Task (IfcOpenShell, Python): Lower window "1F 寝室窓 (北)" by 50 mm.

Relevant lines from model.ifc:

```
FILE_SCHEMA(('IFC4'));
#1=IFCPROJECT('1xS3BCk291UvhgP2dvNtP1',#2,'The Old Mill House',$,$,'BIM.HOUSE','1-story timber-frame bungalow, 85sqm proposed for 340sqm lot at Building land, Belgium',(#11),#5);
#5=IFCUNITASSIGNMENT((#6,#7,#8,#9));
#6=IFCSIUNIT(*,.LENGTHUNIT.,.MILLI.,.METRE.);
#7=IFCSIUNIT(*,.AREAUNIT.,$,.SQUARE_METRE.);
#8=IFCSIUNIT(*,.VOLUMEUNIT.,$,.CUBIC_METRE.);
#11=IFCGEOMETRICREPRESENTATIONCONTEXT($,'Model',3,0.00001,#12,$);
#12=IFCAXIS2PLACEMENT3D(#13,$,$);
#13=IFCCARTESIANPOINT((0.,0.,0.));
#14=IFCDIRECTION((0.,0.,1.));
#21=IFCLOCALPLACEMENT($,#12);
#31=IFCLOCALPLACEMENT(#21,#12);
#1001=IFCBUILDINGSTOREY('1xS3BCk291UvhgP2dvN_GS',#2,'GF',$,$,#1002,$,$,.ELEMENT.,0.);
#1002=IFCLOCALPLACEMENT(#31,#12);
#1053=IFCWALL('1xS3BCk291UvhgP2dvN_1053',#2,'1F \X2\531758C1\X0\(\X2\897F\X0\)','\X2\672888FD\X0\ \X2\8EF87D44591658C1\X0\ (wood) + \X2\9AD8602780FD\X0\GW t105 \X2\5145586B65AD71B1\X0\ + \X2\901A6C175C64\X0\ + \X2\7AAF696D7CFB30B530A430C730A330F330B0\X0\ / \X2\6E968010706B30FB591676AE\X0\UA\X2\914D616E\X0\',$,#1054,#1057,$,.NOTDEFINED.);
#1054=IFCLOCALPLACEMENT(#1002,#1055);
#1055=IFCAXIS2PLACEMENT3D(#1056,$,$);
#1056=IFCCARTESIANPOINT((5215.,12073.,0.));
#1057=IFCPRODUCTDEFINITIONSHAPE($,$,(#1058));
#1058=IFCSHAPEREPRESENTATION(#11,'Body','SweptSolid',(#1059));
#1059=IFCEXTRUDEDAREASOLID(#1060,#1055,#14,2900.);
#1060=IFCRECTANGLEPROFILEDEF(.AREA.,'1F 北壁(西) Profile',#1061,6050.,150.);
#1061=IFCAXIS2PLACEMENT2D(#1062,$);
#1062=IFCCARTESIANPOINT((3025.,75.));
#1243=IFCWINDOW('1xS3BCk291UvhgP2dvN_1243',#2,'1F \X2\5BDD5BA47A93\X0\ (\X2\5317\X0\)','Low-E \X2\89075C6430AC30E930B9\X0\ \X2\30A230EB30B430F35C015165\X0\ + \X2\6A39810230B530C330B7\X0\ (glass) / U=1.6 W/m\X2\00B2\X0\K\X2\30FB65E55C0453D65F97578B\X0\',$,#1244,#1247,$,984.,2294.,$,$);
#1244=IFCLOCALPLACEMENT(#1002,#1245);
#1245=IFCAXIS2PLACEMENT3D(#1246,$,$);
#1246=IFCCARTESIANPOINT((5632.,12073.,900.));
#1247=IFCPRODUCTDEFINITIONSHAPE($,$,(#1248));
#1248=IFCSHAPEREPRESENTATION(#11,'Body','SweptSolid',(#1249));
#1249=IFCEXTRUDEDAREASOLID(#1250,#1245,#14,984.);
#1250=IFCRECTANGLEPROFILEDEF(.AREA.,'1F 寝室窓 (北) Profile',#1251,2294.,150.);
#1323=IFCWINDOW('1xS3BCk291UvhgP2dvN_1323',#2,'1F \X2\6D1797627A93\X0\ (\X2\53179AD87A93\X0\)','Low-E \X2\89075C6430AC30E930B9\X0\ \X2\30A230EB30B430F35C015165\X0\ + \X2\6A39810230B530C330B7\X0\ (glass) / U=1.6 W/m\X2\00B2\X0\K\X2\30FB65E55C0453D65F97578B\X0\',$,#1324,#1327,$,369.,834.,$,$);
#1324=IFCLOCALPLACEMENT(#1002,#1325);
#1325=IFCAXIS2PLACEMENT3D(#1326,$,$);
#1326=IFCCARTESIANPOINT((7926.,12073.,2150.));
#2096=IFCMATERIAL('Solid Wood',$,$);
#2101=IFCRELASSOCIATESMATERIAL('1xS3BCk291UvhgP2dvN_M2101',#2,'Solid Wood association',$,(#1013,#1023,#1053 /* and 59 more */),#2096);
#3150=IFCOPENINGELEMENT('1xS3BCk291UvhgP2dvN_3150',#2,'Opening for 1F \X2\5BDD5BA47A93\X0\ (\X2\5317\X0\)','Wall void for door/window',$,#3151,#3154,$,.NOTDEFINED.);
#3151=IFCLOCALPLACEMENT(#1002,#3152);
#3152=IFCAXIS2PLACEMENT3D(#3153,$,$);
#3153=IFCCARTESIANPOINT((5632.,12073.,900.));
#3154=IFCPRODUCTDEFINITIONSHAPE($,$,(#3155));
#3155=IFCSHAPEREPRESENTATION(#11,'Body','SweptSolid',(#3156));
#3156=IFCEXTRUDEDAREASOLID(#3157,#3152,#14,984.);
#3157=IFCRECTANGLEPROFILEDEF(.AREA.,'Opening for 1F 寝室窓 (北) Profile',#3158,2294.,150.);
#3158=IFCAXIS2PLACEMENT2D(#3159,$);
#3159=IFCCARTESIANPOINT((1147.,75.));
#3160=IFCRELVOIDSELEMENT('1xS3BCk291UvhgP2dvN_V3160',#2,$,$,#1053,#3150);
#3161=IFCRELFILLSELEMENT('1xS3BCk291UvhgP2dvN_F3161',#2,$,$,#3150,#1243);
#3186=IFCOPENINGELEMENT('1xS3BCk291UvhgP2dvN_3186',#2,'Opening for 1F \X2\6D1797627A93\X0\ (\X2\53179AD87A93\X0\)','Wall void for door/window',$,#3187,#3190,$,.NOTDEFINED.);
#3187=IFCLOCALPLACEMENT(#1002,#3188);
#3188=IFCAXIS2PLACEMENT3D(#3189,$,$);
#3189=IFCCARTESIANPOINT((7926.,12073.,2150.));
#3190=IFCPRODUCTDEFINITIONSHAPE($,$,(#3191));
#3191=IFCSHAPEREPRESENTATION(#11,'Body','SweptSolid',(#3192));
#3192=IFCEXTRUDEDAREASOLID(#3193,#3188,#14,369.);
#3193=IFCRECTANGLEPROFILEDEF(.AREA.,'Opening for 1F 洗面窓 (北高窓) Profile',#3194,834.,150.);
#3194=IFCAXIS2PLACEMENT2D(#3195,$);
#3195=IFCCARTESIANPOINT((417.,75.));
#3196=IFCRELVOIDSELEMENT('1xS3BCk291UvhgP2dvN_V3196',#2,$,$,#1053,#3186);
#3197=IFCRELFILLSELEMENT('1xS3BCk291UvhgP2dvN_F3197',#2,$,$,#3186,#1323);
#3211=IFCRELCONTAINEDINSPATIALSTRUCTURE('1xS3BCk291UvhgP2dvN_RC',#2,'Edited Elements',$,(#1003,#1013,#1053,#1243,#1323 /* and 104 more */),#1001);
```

```python
import numpy as np
import ifcopenshell
import ifcopenshell.api.geometry
import ifcopenshell.util.placement
import ifcopenshell.util.unit

model = ifcopenshell.open("model.ifc")
unit_scale = ifcopenshell.util.unit.calculate_unit_scale(model)

window = model.by_id(1243)
opening = window.FillsVoids[0].RelatingOpeningElement
dz = -0.05 / unit_scale

shift = np.array([0.0, 0.0, dz])
# The window is not placed relative to its opening, so move both.
for product in (opening, window):
    matrix = ifcopenshell.util.placement.get_local_placement(product.ObjectPlacement)
    matrix[:3, 3] += shift
    ifcopenshell.api.geometry.edit_object_placement(model, product=product, matrix=matrix, is_si=False)

print(f"moved by {dz * unit_scale:+.3f} m")

model.write("model_rev.ifc")
```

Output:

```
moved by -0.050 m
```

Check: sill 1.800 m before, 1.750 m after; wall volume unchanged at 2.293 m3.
